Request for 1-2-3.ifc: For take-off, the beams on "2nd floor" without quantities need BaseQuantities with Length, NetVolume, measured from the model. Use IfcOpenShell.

First a look at what the model holds.

```python
import ifcopenshell
import ifcopenshell.util.element
import ifcopenshell.util.unit

model = ifcopenshell.open("1-2-3.ifc")
print(model.schema)
for unit_type in ("LENGTHUNIT", "AREAUNIT", "VOLUMEUNIT"):
    print(unit_type, ifcopenshell.util.unit.calculate_unit_scale(model, unit_type))
storey = next(s for s in model.by_type("IfcBuildingStorey") if s.Name == "2nd floor")
beams = [e for e in ifcopenshell.util.element.get_decomposition(storey) if e.is_a("IfcBeam")]
for e in sorted(beams, key=lambda e: e.id()):
    print(e.id(), e.is_a(), e.Name, list(ifcopenshell.util.element.get_psets(e, qtos_only=True)), sep=" | ")
```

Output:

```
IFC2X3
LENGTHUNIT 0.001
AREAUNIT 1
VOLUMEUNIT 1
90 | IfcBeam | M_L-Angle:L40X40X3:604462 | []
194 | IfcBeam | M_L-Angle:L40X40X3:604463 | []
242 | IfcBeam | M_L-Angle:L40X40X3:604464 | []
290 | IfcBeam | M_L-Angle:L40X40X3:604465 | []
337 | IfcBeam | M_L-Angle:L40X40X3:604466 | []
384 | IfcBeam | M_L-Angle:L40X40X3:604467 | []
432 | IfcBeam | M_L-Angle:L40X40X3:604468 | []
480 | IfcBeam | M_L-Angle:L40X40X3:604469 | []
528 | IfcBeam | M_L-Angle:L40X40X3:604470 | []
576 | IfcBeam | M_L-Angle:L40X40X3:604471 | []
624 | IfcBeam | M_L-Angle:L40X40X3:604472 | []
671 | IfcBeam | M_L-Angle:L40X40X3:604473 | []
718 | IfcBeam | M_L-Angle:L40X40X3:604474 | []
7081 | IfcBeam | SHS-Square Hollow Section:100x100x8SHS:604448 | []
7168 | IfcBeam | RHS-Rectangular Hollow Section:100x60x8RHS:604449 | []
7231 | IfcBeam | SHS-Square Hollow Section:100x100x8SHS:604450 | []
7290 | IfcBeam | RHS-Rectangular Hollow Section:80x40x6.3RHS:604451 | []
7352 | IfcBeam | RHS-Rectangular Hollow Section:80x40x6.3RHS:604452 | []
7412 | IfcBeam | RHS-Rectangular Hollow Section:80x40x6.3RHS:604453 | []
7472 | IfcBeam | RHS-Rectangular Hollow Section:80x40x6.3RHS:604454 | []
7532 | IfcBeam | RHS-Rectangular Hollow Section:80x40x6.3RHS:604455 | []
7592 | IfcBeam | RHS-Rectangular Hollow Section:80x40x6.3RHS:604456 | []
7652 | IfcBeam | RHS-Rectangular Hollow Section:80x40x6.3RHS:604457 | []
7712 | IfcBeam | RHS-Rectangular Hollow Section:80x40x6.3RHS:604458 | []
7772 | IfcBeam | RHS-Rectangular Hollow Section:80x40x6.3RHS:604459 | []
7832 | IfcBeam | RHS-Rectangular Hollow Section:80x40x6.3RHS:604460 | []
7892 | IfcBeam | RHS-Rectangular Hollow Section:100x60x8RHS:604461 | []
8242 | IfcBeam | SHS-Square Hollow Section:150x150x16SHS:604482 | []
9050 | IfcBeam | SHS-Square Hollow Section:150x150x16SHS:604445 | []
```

```python
import ifcopenshell
import ifcopenshell.api.pset
import ifcopenshell.geom
import ifcopenshell.util.element
import ifcopenshell.util.shape
import ifcopenshell.util.unit

model = ifcopenshell.open("1-2-3.ifc")
unit_scale = ifcopenshell.util.unit.calculate_unit_scale(model)
volume_scale = ifcopenshell.util.unit.calculate_unit_scale(model, "VOLUMEUNIT")
settings = ifcopenshell.geom.settings()

storey = next(s for s in model.by_type("IfcBuildingStorey") if s.Name == "2nd floor")
beams = [e for e in ifcopenshell.util.element.get_decomposition(storey) if e.is_a("IfcBeam")]

for e in sorted(beams, key=lambda e: e.id()):
    if ifcopenshell.util.element.get_psets(e, qtos_only=True, should_inherit=False):
        continue
    # Geometry comes back in metres, in the element's own axes.
    shape = ifcopenshell.geom.create_shape(settings, e)
    values = {
        "Length": ifcopenshell.util.shape.get_max_xyz(shape.geometry) / unit_scale,
        "NetVolume": ifcopenshell.util.shape.get_volume(shape.geometry) / volume_scale,
    }
    qto = ifcopenshell.api.pset.add_qto(model, product=e, name="BaseQuantities")
    ifcopenshell.api.pset.edit_qto(model, qto=qto, properties=values)
    print(e.id(), {k: round(v, 3) for k, v in values.items()})

model.write("1-2-3-out.ifc")
```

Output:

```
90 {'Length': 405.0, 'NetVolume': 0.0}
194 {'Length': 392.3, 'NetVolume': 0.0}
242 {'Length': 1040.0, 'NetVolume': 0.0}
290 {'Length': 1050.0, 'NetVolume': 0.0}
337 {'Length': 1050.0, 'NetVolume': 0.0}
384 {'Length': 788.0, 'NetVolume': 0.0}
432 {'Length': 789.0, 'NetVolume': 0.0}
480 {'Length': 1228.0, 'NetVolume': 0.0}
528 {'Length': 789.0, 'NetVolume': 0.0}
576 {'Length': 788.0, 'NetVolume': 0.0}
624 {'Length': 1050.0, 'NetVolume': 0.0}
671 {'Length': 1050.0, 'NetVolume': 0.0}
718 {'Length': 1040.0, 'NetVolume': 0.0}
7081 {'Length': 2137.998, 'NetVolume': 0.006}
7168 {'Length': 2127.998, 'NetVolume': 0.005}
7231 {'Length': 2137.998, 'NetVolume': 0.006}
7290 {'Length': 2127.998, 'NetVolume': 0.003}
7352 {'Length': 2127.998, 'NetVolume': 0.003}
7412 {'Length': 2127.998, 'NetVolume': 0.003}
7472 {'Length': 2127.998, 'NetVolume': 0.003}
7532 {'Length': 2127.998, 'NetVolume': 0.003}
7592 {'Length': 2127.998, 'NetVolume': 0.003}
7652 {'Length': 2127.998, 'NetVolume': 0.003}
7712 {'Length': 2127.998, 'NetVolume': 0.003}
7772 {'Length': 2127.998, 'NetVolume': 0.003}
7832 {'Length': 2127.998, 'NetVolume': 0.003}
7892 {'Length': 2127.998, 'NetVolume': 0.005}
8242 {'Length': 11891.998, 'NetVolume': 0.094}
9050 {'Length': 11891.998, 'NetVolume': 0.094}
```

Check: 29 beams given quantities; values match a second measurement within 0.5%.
